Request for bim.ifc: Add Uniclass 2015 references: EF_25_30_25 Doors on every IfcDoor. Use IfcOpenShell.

First a look at what the model holds.

```python
import ifcopenshell

model = ifcopenshell.open("bim.ifc")
print(model.schema)
print("classifications:", [c.Name for c in model.by_type("IfcClassification")])
for ifc_class in ("IfcDoor", "IfcRoof", "IfcStair", "IfcWall", "IfcWindow"):
    print(ifc_class, len(model.by_type(ifc_class)))
```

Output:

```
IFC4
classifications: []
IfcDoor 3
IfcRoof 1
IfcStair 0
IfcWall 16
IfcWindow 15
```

```python
import ifcopenshell
import ifcopenshell.api.classification

model = ifcopenshell.open("bim.ifc")

system = ifcopenshell.api.classification.add_classification(model, classification="Uniclass 2015")

codes = {
    "IfcDoor": ("EF_25_30_25", "Doors"),
}
for ifc_class, (code, name) in codes.items():
    products = model.by_type(ifc_class)
    ifcopenshell.api.classification.add_reference(
        model, products=products, classification=system, identification=code, name=name
    )
    print(code, len(products))

model.write("bim_edited.ifc")
```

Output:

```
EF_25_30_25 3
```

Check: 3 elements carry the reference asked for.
